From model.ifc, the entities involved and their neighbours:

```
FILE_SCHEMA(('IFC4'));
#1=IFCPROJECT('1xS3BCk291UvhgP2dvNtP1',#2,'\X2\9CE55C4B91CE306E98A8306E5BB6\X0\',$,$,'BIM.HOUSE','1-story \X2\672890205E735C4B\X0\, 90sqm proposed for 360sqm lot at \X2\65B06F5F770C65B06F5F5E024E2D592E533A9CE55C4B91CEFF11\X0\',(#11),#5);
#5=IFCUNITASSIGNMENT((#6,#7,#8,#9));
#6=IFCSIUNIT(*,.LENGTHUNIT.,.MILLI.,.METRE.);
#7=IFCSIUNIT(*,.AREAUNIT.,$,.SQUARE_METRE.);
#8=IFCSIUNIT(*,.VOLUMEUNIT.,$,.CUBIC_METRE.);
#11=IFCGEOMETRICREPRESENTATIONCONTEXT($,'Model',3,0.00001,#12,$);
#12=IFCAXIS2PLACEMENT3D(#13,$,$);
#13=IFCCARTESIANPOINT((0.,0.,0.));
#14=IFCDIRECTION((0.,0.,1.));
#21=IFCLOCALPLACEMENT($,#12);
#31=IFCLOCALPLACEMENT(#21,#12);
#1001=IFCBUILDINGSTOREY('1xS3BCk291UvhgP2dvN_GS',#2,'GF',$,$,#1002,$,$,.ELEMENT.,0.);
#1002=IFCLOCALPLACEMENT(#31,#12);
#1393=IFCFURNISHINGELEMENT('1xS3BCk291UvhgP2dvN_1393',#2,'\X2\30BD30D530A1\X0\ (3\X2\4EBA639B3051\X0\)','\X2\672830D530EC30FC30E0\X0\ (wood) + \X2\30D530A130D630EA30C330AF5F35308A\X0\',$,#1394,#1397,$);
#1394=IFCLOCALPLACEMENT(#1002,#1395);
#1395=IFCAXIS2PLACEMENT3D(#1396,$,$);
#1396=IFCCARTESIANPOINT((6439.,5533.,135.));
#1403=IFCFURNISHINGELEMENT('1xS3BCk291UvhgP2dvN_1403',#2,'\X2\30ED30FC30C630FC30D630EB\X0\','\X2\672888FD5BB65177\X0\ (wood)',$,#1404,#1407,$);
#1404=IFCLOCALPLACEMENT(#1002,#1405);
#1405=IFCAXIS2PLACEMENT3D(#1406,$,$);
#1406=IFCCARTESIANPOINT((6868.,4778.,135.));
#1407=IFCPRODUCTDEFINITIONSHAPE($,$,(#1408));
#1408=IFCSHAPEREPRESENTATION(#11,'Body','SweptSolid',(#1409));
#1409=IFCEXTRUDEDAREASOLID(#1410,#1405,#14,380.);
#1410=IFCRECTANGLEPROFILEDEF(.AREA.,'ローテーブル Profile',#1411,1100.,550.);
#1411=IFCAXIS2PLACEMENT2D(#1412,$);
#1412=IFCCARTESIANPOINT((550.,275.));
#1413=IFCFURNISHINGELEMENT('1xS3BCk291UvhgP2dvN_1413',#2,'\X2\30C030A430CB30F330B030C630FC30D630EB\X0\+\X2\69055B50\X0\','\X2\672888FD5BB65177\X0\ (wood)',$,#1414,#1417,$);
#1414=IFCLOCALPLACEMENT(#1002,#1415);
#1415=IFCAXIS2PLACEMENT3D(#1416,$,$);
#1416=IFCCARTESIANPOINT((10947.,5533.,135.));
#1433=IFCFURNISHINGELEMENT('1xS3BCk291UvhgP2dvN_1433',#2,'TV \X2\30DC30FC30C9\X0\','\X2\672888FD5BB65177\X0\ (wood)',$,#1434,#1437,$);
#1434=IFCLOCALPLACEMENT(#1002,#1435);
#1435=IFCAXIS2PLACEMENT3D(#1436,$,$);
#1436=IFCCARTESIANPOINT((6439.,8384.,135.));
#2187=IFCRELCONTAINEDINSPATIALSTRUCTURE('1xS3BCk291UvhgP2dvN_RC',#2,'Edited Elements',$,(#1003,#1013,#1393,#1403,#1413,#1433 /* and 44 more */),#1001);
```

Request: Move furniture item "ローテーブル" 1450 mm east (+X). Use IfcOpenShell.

```python
import ifcopenshell
import ifcopenshell.api.geometry
import ifcopenshell.util.placement
import ifcopenshell.util.unit

model = ifcopenshell.open("model.ifc")
unit_scale = ifcopenshell.util.unit.calculate_unit_scale(model)

item = model.by_guid("1xS3BCk291UvhgP2dvN_1403")
matrix = ifcopenshell.util.placement.get_local_placement(item.ObjectPlacement)
matrix[0, 3] += 1.45 / unit_scale
ifcopenshell.api.geometry.edit_object_placement(model, product=item, matrix=matrix, is_si=False)

print(ifcopenshell.util.placement.get_local_placement(item.ObjectPlacement).round(3) + 0.0)

model.write("model_v2.ifc")
```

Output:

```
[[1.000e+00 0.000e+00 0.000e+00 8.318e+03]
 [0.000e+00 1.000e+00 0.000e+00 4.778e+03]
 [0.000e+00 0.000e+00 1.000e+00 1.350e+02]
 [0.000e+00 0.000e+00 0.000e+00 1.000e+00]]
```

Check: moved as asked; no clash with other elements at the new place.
